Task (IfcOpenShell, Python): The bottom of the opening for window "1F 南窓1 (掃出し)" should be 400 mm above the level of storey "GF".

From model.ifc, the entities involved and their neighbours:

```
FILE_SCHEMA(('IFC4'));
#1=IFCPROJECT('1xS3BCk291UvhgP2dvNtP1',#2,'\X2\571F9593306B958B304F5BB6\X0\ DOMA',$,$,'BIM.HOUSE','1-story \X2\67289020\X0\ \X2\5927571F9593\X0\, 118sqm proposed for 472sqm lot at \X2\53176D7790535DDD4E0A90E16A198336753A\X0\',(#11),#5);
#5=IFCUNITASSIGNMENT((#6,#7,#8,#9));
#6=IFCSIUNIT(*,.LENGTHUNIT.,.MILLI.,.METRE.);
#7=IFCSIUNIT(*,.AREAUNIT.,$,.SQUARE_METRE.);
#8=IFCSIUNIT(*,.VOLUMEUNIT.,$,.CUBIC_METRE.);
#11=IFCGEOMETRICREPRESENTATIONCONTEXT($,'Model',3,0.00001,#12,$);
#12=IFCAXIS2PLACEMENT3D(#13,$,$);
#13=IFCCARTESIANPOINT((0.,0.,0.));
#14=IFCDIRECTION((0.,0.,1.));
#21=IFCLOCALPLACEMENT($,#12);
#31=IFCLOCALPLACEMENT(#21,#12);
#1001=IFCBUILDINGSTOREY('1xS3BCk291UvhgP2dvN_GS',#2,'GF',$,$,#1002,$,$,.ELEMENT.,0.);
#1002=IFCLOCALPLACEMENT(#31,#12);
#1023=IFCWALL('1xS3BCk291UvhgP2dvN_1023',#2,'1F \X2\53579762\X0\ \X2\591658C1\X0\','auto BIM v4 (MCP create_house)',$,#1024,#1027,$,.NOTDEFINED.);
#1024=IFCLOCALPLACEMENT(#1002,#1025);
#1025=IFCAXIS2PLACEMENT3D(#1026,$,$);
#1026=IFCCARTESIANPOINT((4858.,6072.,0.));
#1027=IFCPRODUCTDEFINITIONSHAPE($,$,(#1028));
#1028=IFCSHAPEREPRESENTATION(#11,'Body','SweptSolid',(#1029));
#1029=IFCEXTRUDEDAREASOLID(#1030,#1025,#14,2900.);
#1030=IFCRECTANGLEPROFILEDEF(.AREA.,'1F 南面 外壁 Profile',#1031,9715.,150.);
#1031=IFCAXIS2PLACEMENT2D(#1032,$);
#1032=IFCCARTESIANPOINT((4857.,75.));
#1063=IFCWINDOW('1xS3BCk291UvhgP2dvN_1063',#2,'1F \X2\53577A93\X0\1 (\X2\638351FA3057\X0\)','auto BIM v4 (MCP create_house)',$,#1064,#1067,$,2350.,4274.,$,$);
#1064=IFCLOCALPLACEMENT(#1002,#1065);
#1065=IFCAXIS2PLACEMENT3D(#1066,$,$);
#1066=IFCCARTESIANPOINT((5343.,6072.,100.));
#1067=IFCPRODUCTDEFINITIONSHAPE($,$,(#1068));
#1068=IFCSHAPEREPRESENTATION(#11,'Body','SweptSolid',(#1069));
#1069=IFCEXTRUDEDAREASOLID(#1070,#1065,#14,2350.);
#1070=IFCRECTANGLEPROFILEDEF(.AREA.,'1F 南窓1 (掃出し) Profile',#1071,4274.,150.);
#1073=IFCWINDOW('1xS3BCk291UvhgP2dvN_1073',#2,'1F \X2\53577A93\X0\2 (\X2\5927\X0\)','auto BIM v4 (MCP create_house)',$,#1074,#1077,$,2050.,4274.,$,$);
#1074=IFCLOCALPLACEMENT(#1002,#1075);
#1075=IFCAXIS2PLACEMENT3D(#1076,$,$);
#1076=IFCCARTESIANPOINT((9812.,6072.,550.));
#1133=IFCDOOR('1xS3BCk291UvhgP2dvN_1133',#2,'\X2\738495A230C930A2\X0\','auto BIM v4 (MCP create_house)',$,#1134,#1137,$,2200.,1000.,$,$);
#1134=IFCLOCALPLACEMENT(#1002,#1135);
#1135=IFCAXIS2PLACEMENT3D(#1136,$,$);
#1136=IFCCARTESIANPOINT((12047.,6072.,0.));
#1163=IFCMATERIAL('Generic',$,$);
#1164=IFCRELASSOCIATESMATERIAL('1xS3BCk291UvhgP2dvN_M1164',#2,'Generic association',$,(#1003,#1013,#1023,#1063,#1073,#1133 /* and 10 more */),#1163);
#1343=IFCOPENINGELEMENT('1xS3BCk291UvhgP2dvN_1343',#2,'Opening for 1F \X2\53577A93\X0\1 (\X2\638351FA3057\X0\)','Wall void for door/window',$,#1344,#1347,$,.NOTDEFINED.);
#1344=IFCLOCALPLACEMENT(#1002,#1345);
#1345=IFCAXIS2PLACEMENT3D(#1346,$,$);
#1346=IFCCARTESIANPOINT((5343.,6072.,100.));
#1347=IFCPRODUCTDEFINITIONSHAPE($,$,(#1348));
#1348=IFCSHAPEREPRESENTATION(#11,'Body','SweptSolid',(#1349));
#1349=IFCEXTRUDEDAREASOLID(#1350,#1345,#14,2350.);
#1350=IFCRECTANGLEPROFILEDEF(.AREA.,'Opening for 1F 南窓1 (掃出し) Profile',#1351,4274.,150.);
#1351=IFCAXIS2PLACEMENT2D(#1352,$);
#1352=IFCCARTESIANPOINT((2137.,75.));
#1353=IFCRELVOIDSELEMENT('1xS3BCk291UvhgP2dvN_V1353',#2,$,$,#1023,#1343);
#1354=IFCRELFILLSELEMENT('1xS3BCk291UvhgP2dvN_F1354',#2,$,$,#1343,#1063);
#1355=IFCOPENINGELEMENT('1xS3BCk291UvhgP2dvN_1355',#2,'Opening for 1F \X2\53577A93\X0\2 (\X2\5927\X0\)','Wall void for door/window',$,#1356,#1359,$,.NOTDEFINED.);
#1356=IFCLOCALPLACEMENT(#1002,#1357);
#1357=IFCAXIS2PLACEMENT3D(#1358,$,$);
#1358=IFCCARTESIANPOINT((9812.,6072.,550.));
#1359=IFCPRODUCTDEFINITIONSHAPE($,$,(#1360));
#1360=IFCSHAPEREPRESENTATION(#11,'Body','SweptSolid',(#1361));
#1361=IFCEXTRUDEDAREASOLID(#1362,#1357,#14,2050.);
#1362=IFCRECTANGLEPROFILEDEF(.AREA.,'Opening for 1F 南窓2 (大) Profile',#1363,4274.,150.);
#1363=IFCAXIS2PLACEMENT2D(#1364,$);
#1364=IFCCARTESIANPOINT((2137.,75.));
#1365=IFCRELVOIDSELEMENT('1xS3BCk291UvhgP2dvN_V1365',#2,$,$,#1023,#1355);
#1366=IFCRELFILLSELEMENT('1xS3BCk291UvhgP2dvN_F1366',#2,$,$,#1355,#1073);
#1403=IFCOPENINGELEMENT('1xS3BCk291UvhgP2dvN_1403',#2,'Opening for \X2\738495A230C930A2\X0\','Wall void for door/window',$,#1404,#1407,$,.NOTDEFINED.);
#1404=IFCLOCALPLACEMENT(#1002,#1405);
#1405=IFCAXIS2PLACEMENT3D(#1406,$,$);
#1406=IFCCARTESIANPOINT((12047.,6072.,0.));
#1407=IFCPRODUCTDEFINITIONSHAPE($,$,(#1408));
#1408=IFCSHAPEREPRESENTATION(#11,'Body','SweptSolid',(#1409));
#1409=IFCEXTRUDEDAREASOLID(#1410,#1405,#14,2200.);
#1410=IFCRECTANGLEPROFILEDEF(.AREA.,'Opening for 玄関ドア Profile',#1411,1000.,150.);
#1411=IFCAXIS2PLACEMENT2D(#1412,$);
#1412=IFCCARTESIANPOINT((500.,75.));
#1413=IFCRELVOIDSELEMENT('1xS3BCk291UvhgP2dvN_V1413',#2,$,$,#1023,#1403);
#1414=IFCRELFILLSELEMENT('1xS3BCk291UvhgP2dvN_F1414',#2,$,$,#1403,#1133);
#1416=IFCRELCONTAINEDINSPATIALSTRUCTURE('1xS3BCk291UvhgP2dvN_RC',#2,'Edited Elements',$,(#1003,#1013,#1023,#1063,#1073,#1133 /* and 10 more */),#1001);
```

```python
import numpy as np
import ifcopenshell
import ifcopenshell.api.geometry
import ifcopenshell.geom
import ifcopenshell.util.element
import ifcopenshell.util.placement
import ifcopenshell.util.shape
import ifcopenshell.util.unit

model = ifcopenshell.open("model.ifc")
unit_scale = ifcopenshell.util.unit.calculate_unit_scale(model)

window = model.by_guid("1xS3BCk291UvhgP2dvN_1063")
opening = window.FillsVoids[0].RelatingOpeningElement
storey = ifcopenshell.util.element.get_container(window, ifc_class="IfcBuildingStorey")
level = ifcopenshell.util.placement.get_local_placement(storey.ObjectPlacement)[2, 3]

# The opening's origin need not be at the sill, so measure its lowest point.
shape = ifcopenshell.geom.create_shape(ifcopenshell.geom.settings(), opening)
bottom = ifcopenshell.util.shape.get_shape_bottom_elevation(shape, shape.geometry) / unit_scale
dz = level + 0.4 / unit_scale - bottom

shift = np.array([0.0, 0.0, dz])
# The window is not placed relative to its opening, so move both.
for product in (opening, window):
    matrix = ifcopenshell.util.placement.get_local_placement(product.ObjectPlacement)
    matrix[:3, 3] += shift
    ifcopenshell.api.geometry.edit_object_placement(model, product=product, matrix=matrix, is_si=False)

print(f"moved by {dz * unit_scale:+.3f} m")

model.write("model-out.ifc")
```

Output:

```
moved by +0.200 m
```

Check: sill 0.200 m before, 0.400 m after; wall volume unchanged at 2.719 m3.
